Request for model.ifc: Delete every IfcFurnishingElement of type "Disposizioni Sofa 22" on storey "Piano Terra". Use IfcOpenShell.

First a look at what the model holds.

```python
import ifcopenshell
import ifcopenshell.util.element

model = ifcopenshell.open("model.ifc")
print(model.schema)
storey = next(s for s in model.by_type("IfcBuildingStorey") if s.Name == "Piano Terra")
furniture = [e for e in ifcopenshell.util.element.get_decomposition(storey) if e.is_a("IfcFurnishingElement")]
seen = {}
for e in furniture:
    element_type = ifcopenshell.util.element.get_type(e)
    name = element_type.Name if element_type not in (None, e) else None
    seen[name] = seen.get(name, 0) + 1
for name, count in sorted(seen.items(), key=str):
    print(count, "x", name)
```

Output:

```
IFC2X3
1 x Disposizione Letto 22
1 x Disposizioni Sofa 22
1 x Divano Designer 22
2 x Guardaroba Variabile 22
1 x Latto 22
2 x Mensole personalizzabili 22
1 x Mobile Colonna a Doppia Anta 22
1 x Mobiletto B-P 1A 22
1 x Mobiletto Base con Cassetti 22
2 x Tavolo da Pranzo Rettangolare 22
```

```python
import ifcopenshell
import ifcopenshell.api.root
import ifcopenshell.util.element

model = ifcopenshell.open("model.ifc")

storey = next(s for s in model.by_type("IfcBuildingStorey") if s.Name == "Piano Terra")
furniture = [e for e in ifcopenshell.util.element.get_decomposition(storey) if e.is_a("IfcFurnishingElement")]
targets = [e for e in furniture if (t := ifcopenshell.util.element.get_type(e)) not in (None, e) and t.Name == "Disposizioni Sofa 22"]

for e in targets:
    ifcopenshell.api.root.remove_product(model, product=e)
print(len(targets), "removed")

model.write("model-out.ifc")
```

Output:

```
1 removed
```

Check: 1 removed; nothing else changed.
